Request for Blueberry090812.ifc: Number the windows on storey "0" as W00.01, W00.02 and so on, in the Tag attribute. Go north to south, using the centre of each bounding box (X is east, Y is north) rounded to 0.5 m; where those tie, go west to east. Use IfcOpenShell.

First a look at what the model holds.

```python
import ifcopenshell
import ifcopenshell.util.element
import ifcopenshell.util.placement

model = ifcopenshell.open("Blueberry090812.ifc")
print(model.schema)
storey = next(s for s in model.by_type("IfcBuildingStorey") if s.Name == "0")
windows = [e for e in ifcopenshell.util.element.get_decomposition(storey) if e.is_a("IfcWindow")]
for e in sorted(windows, key=lambda e: e.id()):
    origin = ifcopenshell.util.placement.get_local_placement(e.ObjectPlacement)[:3, 3]
    print(e.id(), e.Tag, e.Name, origin.round(2) + 0.0, sep=" | ")
```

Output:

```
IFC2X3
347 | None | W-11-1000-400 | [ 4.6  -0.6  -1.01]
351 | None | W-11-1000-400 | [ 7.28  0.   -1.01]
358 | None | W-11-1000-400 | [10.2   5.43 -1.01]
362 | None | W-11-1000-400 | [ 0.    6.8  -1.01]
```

```python
import ifcopenshell
import ifcopenshell.geom
import ifcopenshell.util.element
import ifcopenshell.util.shape

model = ifcopenshell.open("Blueberry090812.ifc")
settings = ifcopenshell.geom.settings()
settings.set("use-world-coords", True)


def centre(element):
    shape = ifcopenshell.geom.create_shape(settings, element)
    return ifcopenshell.util.shape.get_bbox_centroid(shape.geometry)


storey = next(s for s in model.by_type("IfcBuildingStorey") if s.Name == "0")
windows = [e for e in ifcopenshell.util.element.get_decomposition(storey) if e.is_a("IfcWindow")]

# Insertion points can sit at a corner or the storey origin, so sort by the geometry (in metres).
centres = {e: centre(e) for e in windows}
windows.sort(key=lambda e: (-round(centres[e][1] / 0.5), centres[e][0]))

for i, e in enumerate(windows, start=1):
    number = f"W00.{i:02d}"
    e.Tag = number
    print(e.id(), number)

model.write("Blueberry090812_rev.ifc")
```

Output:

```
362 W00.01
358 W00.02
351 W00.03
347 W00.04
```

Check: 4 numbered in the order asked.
